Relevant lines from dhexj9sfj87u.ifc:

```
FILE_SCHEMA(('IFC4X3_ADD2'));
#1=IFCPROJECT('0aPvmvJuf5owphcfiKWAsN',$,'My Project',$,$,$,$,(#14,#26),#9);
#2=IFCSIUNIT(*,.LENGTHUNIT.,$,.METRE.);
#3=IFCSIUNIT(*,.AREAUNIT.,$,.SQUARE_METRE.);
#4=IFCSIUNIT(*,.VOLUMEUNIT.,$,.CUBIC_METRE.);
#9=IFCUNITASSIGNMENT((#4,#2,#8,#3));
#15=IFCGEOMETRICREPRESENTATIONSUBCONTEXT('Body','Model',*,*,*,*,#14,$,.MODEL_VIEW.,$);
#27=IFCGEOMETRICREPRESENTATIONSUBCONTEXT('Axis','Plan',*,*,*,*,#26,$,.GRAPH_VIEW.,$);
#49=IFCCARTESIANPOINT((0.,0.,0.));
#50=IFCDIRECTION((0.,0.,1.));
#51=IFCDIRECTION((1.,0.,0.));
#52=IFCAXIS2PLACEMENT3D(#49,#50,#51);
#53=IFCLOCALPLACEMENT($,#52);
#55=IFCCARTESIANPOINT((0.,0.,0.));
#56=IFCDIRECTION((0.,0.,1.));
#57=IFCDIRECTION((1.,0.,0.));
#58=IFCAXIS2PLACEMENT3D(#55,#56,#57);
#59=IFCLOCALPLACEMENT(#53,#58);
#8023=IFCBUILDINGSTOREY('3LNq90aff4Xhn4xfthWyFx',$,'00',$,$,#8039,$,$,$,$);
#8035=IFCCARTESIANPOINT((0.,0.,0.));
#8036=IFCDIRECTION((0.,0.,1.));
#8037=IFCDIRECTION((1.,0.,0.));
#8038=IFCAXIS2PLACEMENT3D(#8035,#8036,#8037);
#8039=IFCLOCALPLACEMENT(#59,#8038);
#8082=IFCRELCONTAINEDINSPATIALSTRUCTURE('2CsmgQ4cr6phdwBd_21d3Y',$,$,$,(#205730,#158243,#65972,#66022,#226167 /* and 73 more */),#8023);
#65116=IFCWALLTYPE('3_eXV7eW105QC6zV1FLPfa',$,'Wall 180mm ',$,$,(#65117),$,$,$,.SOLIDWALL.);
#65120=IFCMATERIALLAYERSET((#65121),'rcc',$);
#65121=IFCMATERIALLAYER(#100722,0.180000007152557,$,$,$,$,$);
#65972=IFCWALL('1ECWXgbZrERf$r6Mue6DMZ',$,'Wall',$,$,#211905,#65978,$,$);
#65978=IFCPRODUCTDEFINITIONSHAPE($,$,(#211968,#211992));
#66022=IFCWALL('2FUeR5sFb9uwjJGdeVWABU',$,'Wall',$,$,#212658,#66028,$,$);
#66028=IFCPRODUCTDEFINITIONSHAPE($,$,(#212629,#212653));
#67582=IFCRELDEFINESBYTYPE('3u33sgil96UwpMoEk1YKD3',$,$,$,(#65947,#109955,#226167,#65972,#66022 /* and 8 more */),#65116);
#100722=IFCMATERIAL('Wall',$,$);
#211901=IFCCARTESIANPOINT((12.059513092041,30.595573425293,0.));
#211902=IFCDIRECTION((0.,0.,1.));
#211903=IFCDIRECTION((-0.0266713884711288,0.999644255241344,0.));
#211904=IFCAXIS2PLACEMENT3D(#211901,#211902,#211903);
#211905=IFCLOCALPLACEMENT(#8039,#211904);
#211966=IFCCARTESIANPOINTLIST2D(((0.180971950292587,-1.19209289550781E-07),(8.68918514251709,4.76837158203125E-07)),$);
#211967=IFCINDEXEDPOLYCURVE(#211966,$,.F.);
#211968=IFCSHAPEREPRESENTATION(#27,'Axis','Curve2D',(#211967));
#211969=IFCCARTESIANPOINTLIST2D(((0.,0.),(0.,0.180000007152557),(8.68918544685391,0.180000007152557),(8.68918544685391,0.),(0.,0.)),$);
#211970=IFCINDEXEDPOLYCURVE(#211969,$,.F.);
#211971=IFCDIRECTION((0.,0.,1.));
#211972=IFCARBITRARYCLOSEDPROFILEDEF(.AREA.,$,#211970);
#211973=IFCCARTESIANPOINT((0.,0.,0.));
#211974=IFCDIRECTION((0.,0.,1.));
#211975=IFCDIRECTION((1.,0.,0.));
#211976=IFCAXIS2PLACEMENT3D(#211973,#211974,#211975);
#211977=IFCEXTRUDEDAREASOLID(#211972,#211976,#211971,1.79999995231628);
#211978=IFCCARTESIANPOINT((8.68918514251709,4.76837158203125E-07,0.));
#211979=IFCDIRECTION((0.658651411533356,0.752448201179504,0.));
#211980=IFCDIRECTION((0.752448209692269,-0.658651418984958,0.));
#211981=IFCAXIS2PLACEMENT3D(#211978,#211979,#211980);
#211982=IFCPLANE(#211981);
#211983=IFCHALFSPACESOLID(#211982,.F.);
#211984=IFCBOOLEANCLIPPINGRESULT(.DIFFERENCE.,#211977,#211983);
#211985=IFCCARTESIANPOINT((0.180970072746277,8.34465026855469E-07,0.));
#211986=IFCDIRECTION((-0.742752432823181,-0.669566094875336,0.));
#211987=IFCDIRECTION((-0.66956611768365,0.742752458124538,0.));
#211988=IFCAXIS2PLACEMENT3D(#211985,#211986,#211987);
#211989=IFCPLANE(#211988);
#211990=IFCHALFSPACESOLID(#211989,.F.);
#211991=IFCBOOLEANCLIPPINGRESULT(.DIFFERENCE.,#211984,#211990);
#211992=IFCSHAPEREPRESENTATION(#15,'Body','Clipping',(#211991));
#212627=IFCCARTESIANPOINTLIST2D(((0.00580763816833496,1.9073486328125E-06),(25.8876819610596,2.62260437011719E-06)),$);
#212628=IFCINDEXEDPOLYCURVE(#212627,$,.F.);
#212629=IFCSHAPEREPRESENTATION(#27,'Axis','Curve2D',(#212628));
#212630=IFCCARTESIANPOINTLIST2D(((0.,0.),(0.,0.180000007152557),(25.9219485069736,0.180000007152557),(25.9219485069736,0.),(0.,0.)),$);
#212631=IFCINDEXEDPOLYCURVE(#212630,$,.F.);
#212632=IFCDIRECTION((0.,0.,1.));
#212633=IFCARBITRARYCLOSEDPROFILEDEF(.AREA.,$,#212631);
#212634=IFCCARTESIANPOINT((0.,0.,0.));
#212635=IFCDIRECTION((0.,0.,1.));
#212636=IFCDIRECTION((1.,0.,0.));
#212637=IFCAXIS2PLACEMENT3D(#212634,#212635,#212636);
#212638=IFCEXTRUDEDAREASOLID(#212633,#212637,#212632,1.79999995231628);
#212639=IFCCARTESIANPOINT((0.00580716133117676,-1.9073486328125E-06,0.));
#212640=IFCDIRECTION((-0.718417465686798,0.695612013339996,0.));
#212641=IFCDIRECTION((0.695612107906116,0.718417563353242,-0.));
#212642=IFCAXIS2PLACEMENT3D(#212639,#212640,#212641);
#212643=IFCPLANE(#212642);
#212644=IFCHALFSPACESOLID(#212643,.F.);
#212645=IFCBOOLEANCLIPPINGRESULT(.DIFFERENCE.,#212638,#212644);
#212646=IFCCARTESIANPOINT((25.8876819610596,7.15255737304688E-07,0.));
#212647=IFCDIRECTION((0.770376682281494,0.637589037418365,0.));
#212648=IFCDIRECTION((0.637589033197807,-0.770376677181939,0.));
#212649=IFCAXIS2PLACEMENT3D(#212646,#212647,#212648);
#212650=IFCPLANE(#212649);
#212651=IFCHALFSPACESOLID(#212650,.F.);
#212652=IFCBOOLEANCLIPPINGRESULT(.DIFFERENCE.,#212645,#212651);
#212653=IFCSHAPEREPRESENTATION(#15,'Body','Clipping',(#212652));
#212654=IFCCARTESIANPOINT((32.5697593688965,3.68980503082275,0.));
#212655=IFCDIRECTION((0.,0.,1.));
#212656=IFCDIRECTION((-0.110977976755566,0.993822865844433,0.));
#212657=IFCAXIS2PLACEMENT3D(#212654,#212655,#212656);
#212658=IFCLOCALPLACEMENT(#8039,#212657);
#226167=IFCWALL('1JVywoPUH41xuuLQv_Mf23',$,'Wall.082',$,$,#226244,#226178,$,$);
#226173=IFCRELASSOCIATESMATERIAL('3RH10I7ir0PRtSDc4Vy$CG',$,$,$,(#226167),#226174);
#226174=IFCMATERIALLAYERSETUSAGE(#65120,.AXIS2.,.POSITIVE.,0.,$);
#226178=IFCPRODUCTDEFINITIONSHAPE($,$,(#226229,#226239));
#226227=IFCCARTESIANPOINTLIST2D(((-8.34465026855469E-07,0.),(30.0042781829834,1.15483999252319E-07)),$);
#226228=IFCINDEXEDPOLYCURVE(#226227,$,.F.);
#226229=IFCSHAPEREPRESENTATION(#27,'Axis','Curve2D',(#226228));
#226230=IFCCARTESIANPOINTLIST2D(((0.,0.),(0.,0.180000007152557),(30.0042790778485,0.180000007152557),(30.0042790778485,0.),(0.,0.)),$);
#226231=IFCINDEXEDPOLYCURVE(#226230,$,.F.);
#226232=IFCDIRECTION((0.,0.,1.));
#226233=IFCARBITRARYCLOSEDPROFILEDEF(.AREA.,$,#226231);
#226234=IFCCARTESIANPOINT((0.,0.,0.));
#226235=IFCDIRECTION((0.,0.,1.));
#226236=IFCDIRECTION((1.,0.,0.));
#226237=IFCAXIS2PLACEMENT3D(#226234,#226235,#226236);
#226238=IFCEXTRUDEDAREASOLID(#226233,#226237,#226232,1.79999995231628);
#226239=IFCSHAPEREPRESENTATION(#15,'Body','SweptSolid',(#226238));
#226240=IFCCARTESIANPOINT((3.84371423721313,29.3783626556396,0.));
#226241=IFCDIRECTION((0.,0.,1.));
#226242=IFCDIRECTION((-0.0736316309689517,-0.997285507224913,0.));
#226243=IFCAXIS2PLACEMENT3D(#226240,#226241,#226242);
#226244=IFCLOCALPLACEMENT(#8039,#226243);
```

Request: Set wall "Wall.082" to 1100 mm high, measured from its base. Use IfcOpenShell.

```python
import ifcopenshell
import ifcopenshell.geom
import ifcopenshell.util.representation
import ifcopenshell.util.shape
import ifcopenshell.util.unit

model = ifcopenshell.open("dhexj9sfj87u.ifc")
unit_scale = ifcopenshell.util.unit.calculate_unit_scale(model)
settings = ifcopenshell.geom.settings()


def volume(element):
    """Net volume in cubic metres, openings subtracted."""
    shape = ifcopenshell.geom.create_shape(settings, element)
    return ifcopenshell.util.shape.get_volume(shape.geometry)


wall = model.by_guid("1JVywoPUH41xuuLQv_Mf23")
before = volume(wall)

body = ifcopenshell.util.representation.get_representation(wall, "Model", "Body")
solid = body.Items[0]
old_height = solid.Depth
solid.Depth = 1.1 / unit_scale
after = volume(wall)

print(f"height {old_height:g} -> {solid.Depth:g}, volume {before:.3f} -> {after:.3f} m3")

model.write("dhexj9sfj87u_rev.ifc")
```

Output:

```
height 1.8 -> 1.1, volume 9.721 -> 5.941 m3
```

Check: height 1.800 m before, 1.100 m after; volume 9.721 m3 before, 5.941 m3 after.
